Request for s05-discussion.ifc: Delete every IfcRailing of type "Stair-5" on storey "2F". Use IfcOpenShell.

First a look at what the model holds.

```python
import ifcopenshell
import ifcopenshell.util.element

model = ifcopenshell.open("s05-discussion.ifc")
print(model.schema)
storey = next(s for s in model.by_type("IfcBuildingStorey") if s.Name == "2F")
railings = [e for e in ifcopenshell.util.element.get_decomposition(storey) if e.is_a("IfcRailing")]
seen = {}
for e in railings:
    element_type = ifcopenshell.util.element.get_type(e)
    name = element_type.Name if element_type not in (None, e) else None
    seen[name] = seen.get(name, 0) + 1
for name, count in sorted(seen.items(), key=str):
    print(count, "x", name)
```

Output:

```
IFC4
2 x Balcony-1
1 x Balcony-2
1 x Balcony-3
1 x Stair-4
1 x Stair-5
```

```python
import ifcopenshell
import ifcopenshell.api.root
import ifcopenshell.util.element

model = ifcopenshell.open("s05-discussion.ifc")

storey = next(s for s in model.by_type("IfcBuildingStorey") if s.Name == "2F")
railings = [e for e in ifcopenshell.util.element.get_decomposition(storey) if e.is_a("IfcRailing")]
targets = [e for e in railings if (t := ifcopenshell.util.element.get_type(e)) not in (None, e) and t.Name == "Stair-5"]

for e in targets:
    ifcopenshell.api.root.remove_product(model, product=e)
print(len(targets), "removed")

model.write("s05-discussion_v2.ifc")
```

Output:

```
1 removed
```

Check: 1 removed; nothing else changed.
